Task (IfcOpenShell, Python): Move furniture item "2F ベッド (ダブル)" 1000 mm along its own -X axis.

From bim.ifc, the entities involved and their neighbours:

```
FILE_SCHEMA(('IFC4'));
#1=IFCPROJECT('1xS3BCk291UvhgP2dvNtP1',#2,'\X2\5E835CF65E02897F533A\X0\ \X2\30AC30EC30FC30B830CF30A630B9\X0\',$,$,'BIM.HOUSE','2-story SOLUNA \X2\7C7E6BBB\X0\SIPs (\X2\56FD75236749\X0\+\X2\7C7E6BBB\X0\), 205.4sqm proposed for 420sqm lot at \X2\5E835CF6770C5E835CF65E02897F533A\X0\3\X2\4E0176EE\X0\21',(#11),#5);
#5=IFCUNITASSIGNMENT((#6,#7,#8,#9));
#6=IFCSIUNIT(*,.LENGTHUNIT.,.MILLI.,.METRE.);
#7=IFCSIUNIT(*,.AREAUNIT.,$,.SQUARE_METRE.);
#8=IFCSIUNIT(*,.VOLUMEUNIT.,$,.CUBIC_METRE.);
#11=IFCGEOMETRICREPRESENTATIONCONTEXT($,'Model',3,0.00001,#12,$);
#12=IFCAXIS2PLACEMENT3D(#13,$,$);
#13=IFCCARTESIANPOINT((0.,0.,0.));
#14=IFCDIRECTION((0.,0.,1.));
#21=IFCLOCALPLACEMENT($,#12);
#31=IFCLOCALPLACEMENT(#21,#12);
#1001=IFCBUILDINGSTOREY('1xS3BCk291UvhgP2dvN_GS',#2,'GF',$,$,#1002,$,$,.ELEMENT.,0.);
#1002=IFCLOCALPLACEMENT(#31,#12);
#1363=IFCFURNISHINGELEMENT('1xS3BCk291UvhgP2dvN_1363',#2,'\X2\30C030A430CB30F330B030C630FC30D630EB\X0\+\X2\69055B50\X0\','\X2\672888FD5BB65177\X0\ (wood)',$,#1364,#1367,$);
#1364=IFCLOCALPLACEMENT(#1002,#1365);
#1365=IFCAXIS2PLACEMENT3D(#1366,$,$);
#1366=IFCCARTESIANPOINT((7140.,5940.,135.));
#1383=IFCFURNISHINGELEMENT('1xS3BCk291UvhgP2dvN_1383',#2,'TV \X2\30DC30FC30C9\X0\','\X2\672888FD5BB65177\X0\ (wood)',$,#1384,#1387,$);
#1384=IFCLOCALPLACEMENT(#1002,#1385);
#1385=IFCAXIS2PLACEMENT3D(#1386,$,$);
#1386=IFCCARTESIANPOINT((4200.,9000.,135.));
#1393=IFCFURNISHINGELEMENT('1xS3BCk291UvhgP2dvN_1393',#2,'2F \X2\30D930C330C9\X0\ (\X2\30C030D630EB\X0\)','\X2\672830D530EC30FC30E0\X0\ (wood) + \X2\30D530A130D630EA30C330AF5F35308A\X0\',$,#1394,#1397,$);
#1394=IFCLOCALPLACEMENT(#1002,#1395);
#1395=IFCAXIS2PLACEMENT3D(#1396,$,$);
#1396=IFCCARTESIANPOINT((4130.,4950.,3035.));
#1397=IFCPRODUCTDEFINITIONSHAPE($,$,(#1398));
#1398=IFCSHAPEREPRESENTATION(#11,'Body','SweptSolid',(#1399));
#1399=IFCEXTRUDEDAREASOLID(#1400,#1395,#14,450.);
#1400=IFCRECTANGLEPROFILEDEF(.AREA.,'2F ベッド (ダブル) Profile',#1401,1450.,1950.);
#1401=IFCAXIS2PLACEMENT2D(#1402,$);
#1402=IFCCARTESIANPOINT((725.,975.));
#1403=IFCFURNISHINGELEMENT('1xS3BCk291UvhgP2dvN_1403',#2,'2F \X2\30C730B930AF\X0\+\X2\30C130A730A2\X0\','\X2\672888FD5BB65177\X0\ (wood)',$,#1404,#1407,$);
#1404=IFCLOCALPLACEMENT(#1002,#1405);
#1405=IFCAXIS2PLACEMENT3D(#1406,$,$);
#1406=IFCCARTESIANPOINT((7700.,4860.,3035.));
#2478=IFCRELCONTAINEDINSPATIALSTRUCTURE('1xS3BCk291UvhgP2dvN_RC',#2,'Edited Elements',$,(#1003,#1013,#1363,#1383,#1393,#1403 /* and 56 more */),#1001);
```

```python
import ifcopenshell
import ifcopenshell.api.geometry
import ifcopenshell.util.placement

model = ifcopenshell.open("bim.ifc")

item = model.by_guid("1xS3BCk291UvhgP2dvN_1393")
matrix = ifcopenshell.util.placement.get_local_placement(item.ObjectPlacement)
matrix[:3, 3] -= matrix[:3, 0] * 1000.0
ifcopenshell.api.geometry.edit_object_placement(model, product=item, matrix=matrix, is_si=False)

print(ifcopenshell.util.placement.get_local_placement(item.ObjectPlacement).round(3) + 0.0)

model.write("bim_updated.ifc")
```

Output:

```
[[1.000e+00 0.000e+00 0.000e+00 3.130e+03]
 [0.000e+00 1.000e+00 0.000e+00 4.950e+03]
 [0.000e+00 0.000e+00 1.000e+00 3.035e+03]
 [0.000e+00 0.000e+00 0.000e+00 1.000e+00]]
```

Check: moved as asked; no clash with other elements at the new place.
